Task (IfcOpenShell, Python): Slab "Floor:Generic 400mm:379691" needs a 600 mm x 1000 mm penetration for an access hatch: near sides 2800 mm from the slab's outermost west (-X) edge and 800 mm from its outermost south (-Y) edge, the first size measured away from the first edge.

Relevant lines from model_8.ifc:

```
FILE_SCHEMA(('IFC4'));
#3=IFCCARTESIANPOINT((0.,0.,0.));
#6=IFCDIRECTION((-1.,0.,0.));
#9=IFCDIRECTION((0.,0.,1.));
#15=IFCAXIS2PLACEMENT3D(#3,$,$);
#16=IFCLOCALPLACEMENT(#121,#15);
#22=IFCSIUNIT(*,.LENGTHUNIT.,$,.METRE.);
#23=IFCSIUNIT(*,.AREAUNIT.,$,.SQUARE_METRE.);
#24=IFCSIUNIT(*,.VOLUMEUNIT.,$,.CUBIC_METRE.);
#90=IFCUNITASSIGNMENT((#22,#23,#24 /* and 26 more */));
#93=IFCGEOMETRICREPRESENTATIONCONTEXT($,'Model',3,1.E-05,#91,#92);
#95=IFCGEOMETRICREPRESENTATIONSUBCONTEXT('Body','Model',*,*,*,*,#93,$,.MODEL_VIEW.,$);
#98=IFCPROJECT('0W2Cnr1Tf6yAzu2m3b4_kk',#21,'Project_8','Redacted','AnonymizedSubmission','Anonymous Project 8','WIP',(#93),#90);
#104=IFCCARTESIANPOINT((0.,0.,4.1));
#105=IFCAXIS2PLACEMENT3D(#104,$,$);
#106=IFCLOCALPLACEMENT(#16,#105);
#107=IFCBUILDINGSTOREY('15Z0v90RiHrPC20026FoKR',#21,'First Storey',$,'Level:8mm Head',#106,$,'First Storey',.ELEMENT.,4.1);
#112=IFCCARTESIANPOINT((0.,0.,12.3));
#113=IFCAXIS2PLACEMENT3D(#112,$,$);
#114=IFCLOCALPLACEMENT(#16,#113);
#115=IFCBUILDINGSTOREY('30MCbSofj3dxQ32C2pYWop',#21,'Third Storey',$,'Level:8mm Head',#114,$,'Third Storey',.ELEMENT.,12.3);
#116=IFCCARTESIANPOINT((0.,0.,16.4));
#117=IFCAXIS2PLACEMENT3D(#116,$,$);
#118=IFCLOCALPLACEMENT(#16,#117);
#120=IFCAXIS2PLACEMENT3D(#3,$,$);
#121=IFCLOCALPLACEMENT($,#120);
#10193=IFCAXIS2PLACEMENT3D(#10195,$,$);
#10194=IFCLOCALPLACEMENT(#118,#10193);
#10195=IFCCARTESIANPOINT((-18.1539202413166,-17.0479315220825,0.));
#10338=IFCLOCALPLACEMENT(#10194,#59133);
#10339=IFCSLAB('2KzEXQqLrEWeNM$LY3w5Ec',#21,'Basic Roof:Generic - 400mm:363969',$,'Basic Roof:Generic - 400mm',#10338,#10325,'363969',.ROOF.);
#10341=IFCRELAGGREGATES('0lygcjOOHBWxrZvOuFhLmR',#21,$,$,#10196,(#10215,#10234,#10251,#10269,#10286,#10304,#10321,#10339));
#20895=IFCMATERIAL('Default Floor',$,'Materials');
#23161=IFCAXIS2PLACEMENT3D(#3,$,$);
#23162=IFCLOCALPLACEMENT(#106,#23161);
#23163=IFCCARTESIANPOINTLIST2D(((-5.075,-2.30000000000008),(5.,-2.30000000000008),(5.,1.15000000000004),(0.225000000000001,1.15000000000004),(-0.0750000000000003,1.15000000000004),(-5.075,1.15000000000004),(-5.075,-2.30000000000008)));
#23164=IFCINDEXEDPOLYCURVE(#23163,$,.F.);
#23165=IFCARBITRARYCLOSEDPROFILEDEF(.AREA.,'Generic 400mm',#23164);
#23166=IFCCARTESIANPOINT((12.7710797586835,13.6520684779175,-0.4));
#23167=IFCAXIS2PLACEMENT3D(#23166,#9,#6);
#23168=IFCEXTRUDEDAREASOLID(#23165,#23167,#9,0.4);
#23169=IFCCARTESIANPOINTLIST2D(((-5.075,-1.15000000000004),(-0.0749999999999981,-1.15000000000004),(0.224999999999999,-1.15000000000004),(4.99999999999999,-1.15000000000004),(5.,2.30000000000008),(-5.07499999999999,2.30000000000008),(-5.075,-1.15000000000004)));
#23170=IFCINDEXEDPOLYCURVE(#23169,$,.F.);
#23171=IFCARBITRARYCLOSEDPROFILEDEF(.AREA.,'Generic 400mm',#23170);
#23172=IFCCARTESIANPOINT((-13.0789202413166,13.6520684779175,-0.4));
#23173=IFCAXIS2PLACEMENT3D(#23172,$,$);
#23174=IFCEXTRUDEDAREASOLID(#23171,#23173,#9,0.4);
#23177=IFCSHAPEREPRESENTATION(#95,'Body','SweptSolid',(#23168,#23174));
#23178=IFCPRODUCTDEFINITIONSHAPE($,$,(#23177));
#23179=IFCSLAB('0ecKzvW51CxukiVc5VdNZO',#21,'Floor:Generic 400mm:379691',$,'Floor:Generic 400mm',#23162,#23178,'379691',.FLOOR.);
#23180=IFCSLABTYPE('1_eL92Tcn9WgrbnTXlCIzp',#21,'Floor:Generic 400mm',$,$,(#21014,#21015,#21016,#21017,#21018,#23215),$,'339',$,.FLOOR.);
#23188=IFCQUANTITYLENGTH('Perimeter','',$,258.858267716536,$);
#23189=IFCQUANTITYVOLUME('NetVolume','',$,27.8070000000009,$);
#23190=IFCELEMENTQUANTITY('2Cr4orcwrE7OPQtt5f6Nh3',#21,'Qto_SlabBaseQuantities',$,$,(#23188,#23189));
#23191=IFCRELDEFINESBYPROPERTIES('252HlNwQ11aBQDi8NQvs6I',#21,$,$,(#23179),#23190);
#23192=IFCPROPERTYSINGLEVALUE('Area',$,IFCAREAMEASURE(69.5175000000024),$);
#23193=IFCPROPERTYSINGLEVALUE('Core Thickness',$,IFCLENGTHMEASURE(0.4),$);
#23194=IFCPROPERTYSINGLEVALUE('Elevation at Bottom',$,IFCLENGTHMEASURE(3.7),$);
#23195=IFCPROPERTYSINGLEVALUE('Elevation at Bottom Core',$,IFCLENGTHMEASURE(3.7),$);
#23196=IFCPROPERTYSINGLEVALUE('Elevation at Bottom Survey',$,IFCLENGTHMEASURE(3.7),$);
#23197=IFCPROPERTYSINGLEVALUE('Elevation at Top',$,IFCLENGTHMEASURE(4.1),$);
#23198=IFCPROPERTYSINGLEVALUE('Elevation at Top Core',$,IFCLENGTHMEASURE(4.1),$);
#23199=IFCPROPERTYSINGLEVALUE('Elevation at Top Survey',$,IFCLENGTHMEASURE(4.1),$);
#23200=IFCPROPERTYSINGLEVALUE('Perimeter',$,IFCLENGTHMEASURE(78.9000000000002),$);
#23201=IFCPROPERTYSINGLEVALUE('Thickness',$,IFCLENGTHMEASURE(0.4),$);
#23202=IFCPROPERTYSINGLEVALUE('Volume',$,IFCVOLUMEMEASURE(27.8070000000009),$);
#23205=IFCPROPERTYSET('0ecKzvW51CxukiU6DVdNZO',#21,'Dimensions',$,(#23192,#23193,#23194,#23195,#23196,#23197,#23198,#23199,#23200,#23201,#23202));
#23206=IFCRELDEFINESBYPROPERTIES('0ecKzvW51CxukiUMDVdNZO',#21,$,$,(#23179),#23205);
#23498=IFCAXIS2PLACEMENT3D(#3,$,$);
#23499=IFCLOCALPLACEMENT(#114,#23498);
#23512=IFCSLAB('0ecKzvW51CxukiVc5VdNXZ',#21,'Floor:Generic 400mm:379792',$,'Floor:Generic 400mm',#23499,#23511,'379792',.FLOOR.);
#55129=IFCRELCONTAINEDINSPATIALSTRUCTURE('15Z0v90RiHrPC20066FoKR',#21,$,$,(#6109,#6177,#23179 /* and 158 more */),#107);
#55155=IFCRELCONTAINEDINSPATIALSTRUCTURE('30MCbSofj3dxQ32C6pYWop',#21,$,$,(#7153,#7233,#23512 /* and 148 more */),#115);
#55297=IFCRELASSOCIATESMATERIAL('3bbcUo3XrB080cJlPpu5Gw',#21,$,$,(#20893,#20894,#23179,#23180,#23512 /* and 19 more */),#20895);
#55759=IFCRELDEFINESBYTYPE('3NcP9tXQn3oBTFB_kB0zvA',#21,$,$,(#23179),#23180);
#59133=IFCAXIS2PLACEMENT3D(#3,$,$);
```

```python
import numpy as np
import ifcopenshell
import ifcopenshell.api.feature
import ifcopenshell.api.geometry
import ifcopenshell.api.pset
import ifcopenshell.api.root
import ifcopenshell.geom
import ifcopenshell.util.element
import ifcopenshell.util.placement
import ifcopenshell.util.representation
import ifcopenshell.util.shape
import ifcopenshell.util.unit

model = ifcopenshell.open("model_8.ifc")
unit_scale = ifcopenshell.util.unit.calculate_unit_scale(model)
area_scale = ifcopenshell.util.unit.calculate_unit_scale(model, "AREAUNIT")
volume_scale = ifcopenshell.util.unit.calculate_unit_scale(model, "VOLUMEUNIT")
settings = ifcopenshell.geom.settings()


def volume(element):
    """Net volume in cubic metres, openings subtracted."""
    shape = ifcopenshell.geom.create_shape(settings, element)
    return ifcopenshell.util.shape.get_volume(shape.geometry)


slab = model.by_guid("0ecKzvW51CxukiVc5VdNZO")
before = volume(slab)

# Extent in the slab's own axes, in metres. The edges named are its -X and -Y sides.
slab_shape = ifcopenshell.geom.create_shape(settings, slab)
vertices = ifcopenshell.util.shape.get_vertices(slab_shape.geometry)
x_min, y_min, bottom = vertices.min(axis=0)
top = vertices[:, 2].max()

opening = ifcopenshell.api.root.create_entity(model, ifc_class="IfcOpeningElement", name="Access hatch opening", predefined_type="OPENING")
context = ifcopenshell.util.representation.get_context(model, "Model", "Body", "MODEL_VIEW")
width, depth = 0.6, 1
outline = [(0.0, 0.0), (width, 0.0), (width, depth), (0.0, depth), (0.0, 0.0)]
# Overshoot both faces by 50 mm so the cut is clean.
shape = ifcopenshell.api.geometry.add_slab_representation(
    model, context=context, depth=top - bottom + 0.1, polyline=outline
)
ifcopenshell.api.geometry.assign_representation(model, product=opening, representation=shape)

matrix = ifcopenshell.util.placement.get_local_placement(slab.ObjectPlacement)
matrix[:, 3] = matrix @ np.append(np.array([x_min + 2.8, y_min + 0.8, bottom - 0.05]) / unit_scale, 1.0)
ifcopenshell.api.geometry.edit_object_placement(model, product=opening, matrix=matrix, is_si=False)
ifcopenshell.api.feature.add_feature(model, feature=opening, element=slab)

after = volume(slab)

# Update the slab's stored quantities.
qto = model.by_id(ifcopenshell.util.element.get_pset(slab, "Qto_SlabBaseQuantities", should_inherit=False)["id"])
ifcopenshell.api.pset.edit_qto(model, qto=qto, properties={"NetVolume": after / volume_scale})
pset = model.by_id(ifcopenshell.util.element.get_pset(slab, "Dimensions", should_inherit=False)["id"])
ifcopenshell.api.pset.edit_pset(model, pset=pset, properties={
    "Area": model.create_entity("IfcAreaMeasure", after / (top - bottom) / area_scale),
    "Volume": model.create_entity("IfcVolumeMeasure", after / volume_scale),
})

print(f"slab volume {before:.3f} -> {after:.3f} m3")

model.write("model_8_edited.ifc")
```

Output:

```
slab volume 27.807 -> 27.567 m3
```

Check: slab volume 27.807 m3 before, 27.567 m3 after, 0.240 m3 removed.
